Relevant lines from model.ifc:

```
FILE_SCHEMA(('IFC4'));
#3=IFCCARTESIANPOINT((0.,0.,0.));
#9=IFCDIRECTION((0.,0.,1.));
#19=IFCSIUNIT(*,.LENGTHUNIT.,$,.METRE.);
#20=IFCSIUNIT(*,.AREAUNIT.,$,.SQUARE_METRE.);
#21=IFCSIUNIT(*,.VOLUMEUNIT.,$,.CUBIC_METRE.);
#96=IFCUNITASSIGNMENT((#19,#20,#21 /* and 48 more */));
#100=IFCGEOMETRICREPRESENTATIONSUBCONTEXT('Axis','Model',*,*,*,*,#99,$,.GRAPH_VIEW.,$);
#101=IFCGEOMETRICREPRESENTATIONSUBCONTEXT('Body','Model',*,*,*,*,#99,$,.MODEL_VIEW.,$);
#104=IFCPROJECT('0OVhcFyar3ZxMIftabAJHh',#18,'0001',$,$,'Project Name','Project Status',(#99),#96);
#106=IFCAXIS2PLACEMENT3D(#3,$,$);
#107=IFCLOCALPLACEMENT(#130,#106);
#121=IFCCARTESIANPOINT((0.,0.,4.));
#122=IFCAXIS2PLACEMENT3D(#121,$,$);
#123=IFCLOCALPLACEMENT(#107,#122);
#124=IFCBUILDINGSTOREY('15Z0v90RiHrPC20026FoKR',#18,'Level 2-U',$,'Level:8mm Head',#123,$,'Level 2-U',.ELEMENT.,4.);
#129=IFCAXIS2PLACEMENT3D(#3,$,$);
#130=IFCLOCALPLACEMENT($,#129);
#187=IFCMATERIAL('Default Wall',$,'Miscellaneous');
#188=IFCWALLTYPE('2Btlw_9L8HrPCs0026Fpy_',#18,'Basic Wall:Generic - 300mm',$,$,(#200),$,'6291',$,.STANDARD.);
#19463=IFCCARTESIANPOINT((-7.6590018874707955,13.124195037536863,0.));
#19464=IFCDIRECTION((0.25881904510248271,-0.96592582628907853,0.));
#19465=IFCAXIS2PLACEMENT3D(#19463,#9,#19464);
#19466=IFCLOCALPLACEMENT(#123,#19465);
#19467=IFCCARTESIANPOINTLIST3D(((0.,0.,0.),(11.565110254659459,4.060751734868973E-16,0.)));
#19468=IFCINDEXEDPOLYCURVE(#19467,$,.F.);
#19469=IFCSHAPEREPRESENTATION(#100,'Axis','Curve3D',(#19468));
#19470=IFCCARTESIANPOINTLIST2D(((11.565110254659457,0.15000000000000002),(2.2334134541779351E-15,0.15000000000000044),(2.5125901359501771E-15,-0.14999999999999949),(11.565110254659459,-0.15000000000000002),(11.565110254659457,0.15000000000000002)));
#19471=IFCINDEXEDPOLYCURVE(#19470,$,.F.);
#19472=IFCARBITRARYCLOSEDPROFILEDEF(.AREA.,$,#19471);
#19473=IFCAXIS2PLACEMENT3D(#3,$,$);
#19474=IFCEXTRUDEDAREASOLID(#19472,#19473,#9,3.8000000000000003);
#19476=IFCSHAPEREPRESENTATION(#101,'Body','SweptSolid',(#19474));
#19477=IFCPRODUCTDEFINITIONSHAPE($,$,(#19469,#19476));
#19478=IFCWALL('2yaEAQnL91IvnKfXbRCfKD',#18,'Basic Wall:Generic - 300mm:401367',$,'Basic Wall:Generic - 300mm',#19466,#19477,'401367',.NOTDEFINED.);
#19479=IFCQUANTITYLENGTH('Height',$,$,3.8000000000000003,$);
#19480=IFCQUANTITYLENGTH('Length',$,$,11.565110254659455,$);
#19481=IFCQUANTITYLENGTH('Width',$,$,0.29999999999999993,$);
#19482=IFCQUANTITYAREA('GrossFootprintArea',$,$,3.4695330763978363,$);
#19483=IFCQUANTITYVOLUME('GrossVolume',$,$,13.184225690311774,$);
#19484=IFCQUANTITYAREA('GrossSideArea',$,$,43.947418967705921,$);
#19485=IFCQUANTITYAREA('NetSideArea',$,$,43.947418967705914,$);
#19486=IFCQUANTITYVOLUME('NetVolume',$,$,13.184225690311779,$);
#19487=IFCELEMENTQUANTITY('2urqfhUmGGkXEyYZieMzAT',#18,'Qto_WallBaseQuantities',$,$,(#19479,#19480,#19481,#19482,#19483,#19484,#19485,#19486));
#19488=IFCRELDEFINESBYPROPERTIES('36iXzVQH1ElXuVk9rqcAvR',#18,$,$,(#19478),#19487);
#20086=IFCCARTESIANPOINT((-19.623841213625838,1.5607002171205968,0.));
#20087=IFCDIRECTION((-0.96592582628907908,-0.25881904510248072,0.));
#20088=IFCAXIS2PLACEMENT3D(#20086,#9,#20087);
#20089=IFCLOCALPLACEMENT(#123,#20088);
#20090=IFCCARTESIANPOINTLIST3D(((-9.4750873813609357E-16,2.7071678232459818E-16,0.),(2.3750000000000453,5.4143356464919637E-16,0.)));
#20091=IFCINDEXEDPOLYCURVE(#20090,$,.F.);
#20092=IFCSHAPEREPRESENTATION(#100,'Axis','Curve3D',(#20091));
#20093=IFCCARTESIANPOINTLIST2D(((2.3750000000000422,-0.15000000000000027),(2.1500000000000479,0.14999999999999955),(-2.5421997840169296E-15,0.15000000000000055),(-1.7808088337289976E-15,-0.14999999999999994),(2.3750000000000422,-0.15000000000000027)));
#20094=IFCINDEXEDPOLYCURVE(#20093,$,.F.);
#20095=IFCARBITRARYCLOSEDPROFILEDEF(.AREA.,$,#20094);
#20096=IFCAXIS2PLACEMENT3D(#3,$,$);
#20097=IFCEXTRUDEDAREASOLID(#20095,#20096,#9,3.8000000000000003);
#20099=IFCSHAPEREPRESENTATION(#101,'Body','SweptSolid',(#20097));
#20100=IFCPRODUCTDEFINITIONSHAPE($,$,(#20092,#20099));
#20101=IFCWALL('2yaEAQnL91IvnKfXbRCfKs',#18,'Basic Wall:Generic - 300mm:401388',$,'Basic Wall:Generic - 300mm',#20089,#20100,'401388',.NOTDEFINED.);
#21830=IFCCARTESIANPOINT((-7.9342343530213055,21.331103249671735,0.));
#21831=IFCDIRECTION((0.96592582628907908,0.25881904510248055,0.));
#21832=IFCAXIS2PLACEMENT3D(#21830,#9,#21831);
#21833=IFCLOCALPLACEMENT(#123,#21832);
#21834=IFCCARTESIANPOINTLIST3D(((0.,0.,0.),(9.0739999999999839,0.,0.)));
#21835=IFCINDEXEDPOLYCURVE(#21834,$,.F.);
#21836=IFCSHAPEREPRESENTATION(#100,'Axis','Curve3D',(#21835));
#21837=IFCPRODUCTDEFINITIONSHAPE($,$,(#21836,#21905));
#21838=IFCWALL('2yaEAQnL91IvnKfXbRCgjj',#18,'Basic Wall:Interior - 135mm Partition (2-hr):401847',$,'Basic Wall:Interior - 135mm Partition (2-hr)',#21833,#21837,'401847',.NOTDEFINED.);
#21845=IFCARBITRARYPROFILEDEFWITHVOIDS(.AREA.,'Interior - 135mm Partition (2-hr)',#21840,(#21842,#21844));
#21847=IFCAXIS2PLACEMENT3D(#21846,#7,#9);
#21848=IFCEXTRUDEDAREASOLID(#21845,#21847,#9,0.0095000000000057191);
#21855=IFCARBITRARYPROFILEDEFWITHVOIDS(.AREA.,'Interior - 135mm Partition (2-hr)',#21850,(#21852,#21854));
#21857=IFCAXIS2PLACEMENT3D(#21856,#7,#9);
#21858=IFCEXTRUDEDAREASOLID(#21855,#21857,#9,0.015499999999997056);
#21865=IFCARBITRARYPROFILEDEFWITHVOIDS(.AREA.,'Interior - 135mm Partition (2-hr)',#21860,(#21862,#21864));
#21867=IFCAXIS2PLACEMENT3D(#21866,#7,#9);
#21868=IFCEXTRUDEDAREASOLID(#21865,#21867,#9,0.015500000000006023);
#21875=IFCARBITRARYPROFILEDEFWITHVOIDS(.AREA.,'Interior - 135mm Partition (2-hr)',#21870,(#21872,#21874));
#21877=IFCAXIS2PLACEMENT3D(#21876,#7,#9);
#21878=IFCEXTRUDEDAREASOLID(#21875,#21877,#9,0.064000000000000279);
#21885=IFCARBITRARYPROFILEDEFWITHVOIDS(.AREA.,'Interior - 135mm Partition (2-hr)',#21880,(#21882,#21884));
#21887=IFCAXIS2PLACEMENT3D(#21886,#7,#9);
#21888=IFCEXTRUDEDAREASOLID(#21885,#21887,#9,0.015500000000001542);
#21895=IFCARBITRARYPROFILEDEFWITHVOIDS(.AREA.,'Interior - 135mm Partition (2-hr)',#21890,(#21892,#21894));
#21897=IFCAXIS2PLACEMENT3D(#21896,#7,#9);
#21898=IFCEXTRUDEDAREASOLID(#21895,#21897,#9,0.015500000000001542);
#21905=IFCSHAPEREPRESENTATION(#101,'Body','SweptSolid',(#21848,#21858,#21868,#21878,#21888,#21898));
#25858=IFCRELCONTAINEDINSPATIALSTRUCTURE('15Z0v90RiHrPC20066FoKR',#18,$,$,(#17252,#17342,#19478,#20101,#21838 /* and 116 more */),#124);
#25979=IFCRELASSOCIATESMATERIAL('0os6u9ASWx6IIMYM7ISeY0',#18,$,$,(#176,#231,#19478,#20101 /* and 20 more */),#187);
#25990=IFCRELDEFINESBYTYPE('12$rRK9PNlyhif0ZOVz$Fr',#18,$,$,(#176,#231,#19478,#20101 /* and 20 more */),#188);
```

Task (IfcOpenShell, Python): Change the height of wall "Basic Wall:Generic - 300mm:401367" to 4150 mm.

```python
import ifcopenshell
import ifcopenshell.api.pset
import ifcopenshell.geom
import ifcopenshell.util.element
import ifcopenshell.util.representation
import ifcopenshell.util.shape
import ifcopenshell.util.unit

model = ifcopenshell.open("model.ifc")
unit_scale = ifcopenshell.util.unit.calculate_unit_scale(model)
area_scale = ifcopenshell.util.unit.calculate_unit_scale(model, "AREAUNIT")
volume_scale = ifcopenshell.util.unit.calculate_unit_scale(model, "VOLUMEUNIT")
settings = ifcopenshell.geom.settings()


def volume(element):
    """Net volume in cubic metres, openings subtracted."""
    shape = ifcopenshell.geom.create_shape(settings, element)
    return ifcopenshell.util.shape.get_volume(shape.geometry)


wall = model.by_guid("2yaEAQnL91IvnKfXbRCfKD")
before = volume(wall)

body = ifcopenshell.util.representation.get_representation(wall, "Model", "Body")
solid = body.Items[0]
old_height = solid.Depth
solid.Depth = 4.15
after = volume(wall)
thickness = 0.3  # wall thickness in metres

# Update the stored height, areas and volumes.
qto = model.by_id(ifcopenshell.util.element.get_pset(wall, "Qto_WallBaseQuantities", should_inherit=False)["id"])
ifcopenshell.api.pset.edit_qto(model, qto=qto, properties={
    "Height": solid.Depth,
    "GrossVolume": ifcopenshell.util.element.get_pset(wall, "Qto_WallBaseQuantities", "GrossVolume") * solid.Depth / old_height,
    "GrossSideArea": ifcopenshell.util.element.get_pset(wall, "Qto_WallBaseQuantities", "GrossSideArea") * solid.Depth / old_height,
    "NetSideArea": after / thickness / area_scale,
    "NetVolume": after / volume_scale,
})

print(f"height {old_height:g} -> {solid.Depth:g}, volume {before:.3f} -> {after:.3f} m3")

model.write("model_v2.ifc")
```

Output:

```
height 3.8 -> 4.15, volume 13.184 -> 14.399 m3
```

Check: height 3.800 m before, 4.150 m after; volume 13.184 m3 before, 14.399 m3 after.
